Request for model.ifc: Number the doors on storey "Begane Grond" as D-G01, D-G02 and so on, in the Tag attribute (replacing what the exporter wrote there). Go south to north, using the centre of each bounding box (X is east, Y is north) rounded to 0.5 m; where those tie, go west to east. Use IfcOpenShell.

First a look at what the model holds.

```python
import ifcopenshell
import ifcopenshell.util.element
import ifcopenshell.util.placement

model = ifcopenshell.open("model.ifc")
print(model.schema)
storey = next(s for s in model.by_type("IfcBuildingStorey") if s.Name == "Begane Grond")
doors = [e for e in ifcopenshell.util.element.get_decomposition(storey) if e.is_a("IfcDoor")]
for e in sorted(doors, key=lambda e: e.id()):
    origin = ifcopenshell.util.placement.get_local_placement(e.ObjectPlacement)[:3, 3]
    print(e.id(), e.Tag, e.Name, origin.round(2) + 0.0, sep=" | ")
```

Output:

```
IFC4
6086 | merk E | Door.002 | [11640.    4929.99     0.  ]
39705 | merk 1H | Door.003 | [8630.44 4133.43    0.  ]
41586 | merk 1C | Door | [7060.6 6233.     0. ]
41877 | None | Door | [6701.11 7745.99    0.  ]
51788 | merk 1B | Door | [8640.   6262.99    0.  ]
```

```python
import ifcopenshell
import ifcopenshell.geom
import ifcopenshell.util.element
import ifcopenshell.util.shape

model = ifcopenshell.open("model.ifc")
settings = ifcopenshell.geom.settings()
settings.set("use-world-coords", True)


def centre(element):
    shape = ifcopenshell.geom.create_shape(settings, element)
    return ifcopenshell.util.shape.get_bbox_centroid(shape.geometry)


storey = next(s for s in model.by_type("IfcBuildingStorey") if s.Name == "Begane Grond")
doors = [e for e in ifcopenshell.util.element.get_decomposition(storey) if e.is_a("IfcDoor")]

# Insertion points can sit at a corner or the storey origin, so sort by the geometry (in metres).
centres = {e: centre(e) for e in doors}
doors.sort(key=lambda e: (round(centres[e][1] / 0.5), centres[e][0]))

for i, e in enumerate(doors, start=1):
    number = f"D-G{i:02d}"
    e.Tag = number
    print(e.id(), number)

model.write("model_updated.ifc")
```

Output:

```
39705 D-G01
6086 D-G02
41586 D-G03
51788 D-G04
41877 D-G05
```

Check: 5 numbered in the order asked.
